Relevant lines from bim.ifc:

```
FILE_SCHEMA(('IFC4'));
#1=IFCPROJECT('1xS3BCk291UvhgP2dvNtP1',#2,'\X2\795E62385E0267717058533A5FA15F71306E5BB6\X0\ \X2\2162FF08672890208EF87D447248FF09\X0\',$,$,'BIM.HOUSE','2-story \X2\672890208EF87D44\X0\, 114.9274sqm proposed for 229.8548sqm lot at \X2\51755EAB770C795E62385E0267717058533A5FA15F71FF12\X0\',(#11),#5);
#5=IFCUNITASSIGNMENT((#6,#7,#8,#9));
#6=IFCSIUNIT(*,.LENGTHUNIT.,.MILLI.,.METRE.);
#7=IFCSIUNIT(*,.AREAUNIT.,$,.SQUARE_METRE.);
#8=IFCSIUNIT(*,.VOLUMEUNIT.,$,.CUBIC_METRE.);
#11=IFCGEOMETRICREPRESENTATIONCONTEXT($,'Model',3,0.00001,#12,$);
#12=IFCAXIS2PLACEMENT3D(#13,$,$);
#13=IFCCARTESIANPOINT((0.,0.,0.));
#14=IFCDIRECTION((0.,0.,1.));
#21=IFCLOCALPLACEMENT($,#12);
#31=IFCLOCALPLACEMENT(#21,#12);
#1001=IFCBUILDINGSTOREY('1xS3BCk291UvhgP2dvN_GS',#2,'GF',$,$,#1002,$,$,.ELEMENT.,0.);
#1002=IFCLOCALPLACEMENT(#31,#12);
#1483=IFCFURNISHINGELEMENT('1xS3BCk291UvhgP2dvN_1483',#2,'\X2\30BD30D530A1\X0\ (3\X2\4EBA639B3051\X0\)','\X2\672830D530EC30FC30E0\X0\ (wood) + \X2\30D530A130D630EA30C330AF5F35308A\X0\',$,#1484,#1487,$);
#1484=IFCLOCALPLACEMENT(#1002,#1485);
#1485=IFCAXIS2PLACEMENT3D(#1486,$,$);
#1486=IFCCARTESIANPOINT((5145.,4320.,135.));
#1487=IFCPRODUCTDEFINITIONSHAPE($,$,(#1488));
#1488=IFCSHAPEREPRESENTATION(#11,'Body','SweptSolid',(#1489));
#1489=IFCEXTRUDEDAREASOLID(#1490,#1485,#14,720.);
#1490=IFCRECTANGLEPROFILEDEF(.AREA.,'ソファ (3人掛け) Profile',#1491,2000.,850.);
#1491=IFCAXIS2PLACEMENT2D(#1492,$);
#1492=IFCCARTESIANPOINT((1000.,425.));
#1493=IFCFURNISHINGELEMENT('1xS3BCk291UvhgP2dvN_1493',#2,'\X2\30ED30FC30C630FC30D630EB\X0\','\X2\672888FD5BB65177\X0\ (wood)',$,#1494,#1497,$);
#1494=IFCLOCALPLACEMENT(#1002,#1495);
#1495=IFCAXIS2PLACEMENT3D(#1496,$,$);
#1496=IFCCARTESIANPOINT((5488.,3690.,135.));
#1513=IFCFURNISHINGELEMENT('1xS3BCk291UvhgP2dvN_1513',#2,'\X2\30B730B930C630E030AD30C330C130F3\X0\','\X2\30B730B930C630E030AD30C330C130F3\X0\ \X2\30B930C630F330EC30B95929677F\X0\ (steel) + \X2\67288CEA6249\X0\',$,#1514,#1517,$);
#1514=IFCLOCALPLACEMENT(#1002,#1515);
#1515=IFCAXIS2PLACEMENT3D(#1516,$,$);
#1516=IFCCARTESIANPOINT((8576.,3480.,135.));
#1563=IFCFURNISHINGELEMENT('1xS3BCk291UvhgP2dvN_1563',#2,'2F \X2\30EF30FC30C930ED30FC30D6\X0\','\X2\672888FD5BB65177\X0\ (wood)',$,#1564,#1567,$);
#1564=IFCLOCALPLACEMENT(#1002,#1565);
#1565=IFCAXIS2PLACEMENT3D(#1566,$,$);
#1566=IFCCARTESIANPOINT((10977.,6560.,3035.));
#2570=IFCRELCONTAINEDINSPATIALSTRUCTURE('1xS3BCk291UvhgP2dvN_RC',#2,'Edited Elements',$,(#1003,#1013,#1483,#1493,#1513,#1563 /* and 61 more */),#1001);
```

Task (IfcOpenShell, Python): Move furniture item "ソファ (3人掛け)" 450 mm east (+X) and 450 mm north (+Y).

```python
import ifcopenshell
import ifcopenshell.api.geometry
import ifcopenshell.util.placement

model = ifcopenshell.open("bim.ifc")

item = model.by_id(1483)
matrix = ifcopenshell.util.placement.get_local_placement(item.ObjectPlacement)
matrix[0, 3] += 450.0
matrix[1, 3] += 450.0
ifcopenshell.api.geometry.edit_object_placement(model, product=item, matrix=matrix, is_si=False)

print(ifcopenshell.util.placement.get_local_placement(item.ObjectPlacement).round(3) + 0.0)

model.write("bim_v2.ifc")
```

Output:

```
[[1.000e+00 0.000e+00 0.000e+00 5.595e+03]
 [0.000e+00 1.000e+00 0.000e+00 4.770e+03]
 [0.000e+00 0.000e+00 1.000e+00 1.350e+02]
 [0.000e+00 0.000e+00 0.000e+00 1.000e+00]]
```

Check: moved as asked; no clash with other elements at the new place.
